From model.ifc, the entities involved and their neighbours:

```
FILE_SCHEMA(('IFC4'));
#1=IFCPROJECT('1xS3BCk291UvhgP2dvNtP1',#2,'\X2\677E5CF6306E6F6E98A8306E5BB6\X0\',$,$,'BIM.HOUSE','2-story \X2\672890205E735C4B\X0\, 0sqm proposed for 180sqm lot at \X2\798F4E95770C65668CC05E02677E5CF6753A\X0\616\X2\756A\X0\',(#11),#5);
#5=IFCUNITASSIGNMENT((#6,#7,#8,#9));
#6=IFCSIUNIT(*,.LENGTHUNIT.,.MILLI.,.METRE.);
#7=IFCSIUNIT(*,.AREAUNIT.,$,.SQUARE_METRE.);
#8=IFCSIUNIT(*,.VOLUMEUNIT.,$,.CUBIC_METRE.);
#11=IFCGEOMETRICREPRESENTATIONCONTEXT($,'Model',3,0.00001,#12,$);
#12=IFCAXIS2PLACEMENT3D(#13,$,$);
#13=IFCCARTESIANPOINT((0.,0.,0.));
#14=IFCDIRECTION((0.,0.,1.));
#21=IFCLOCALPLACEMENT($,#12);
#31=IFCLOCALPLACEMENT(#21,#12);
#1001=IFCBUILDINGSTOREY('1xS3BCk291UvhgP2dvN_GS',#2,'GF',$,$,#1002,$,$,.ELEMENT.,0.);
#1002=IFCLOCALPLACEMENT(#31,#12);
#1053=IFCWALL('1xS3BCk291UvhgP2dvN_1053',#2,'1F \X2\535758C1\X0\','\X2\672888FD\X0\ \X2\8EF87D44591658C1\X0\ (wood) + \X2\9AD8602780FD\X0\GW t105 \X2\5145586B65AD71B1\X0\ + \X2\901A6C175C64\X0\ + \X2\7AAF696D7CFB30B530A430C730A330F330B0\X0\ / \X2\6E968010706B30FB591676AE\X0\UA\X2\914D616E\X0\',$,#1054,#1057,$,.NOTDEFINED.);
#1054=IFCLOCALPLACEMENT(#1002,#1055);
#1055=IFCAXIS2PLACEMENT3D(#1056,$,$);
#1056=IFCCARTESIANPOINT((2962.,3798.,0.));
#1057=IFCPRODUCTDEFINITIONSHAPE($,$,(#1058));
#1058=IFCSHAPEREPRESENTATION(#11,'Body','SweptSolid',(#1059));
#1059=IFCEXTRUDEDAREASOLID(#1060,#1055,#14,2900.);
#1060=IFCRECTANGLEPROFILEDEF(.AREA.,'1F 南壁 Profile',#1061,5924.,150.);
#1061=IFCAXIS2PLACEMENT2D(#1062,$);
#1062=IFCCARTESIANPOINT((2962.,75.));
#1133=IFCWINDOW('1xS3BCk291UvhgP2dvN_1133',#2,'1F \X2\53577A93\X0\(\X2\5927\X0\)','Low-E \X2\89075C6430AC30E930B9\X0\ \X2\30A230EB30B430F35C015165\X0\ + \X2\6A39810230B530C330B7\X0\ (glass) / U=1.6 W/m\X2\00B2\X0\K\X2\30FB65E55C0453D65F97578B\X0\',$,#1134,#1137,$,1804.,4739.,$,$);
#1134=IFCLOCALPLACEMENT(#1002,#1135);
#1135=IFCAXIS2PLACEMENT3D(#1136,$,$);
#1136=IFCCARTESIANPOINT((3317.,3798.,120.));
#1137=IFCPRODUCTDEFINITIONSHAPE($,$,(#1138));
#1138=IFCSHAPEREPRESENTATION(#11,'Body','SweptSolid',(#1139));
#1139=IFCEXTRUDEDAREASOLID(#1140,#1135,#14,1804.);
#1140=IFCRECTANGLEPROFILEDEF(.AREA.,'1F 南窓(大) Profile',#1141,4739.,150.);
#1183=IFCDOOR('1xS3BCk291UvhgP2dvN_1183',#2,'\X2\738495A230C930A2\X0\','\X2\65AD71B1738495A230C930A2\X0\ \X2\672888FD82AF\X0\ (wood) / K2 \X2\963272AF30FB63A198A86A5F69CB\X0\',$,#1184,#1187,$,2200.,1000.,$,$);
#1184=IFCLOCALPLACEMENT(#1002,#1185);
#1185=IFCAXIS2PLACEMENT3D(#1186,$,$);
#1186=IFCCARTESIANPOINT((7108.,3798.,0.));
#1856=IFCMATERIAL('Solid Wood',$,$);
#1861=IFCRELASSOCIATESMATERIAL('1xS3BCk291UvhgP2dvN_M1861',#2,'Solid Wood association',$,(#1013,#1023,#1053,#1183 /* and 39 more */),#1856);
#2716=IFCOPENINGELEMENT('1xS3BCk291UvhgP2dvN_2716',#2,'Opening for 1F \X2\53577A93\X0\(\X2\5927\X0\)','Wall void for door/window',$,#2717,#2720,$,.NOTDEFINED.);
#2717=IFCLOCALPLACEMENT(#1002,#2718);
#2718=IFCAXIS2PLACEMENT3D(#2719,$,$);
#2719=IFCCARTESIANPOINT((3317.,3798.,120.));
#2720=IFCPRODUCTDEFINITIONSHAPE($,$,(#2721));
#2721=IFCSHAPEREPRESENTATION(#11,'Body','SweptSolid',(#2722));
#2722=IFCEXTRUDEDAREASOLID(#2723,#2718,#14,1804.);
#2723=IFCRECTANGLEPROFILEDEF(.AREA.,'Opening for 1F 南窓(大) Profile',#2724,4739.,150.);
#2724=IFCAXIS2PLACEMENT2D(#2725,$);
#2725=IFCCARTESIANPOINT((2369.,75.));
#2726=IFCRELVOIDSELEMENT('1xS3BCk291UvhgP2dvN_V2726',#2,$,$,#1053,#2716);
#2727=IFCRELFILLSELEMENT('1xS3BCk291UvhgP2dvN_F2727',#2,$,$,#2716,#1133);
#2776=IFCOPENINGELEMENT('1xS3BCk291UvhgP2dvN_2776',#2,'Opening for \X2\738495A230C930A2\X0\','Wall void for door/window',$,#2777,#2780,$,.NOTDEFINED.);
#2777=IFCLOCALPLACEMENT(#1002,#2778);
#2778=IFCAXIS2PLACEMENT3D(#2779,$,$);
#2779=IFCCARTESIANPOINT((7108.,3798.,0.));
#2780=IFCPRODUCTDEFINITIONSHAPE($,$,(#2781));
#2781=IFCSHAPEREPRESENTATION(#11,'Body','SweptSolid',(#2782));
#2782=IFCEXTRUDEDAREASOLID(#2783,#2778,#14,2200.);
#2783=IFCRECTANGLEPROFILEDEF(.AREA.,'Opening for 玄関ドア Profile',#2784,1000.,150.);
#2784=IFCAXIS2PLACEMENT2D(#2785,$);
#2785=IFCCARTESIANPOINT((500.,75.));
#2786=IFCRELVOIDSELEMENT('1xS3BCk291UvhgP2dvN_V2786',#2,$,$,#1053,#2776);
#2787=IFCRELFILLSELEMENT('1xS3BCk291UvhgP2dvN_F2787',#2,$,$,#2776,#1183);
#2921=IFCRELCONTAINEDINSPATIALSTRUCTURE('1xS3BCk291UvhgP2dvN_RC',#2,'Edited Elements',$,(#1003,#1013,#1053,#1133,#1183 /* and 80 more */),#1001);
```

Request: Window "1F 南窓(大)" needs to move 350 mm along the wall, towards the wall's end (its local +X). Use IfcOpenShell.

```python
import ifcopenshell
import ifcopenshell.api.geometry
import ifcopenshell.util.placement
import ifcopenshell.util.unit

model = ifcopenshell.open("model.ifc")
unit_scale = ifcopenshell.util.unit.calculate_unit_scale(model)

window = model.by_guid("1xS3BCk291UvhgP2dvN_1133")
opening = window.FillsVoids[0].RelatingOpeningElement
wall = opening.VoidsElements[0].RelatingBuildingElement

wall_matrix = ifcopenshell.util.placement.get_local_placement(wall.ObjectPlacement)
shift = wall_matrix[:3, 0] * 0.35 / unit_scale
before = ifcopenshell.util.placement.get_local_placement(window.ObjectPlacement)[:3, 3].copy()

# The window is not placed relative to its opening, so move both.
for product in (opening, window):
    matrix = ifcopenshell.util.placement.get_local_placement(product.ObjectPlacement)
    matrix[:3, 3] += shift
    ifcopenshell.api.geometry.edit_object_placement(model, product=product, matrix=matrix, is_si=False)

after = ifcopenshell.util.placement.get_local_placement(window.ObjectPlacement)[:3, 3]
print("window moved by", (after - before).round(3) + 0.0)

model.write("model_rev.ifc")
```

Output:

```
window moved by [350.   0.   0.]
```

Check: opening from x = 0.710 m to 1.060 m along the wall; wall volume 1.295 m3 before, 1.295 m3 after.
